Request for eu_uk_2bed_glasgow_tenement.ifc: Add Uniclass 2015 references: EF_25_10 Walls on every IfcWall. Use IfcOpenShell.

First a look at what the model holds.

```python
import ifcopenshell

model = ifcopenshell.open("eu_uk_2bed_glasgow_tenement.ifc")
print(model.schema)
print("classifications:", [c.Name for c in model.by_type("IfcClassification")])
for ifc_class in ("IfcDoor", "IfcRoof", "IfcStair", "IfcWall", "IfcWindow"):
    print(ifc_class, len(model.by_type(ifc_class)))
```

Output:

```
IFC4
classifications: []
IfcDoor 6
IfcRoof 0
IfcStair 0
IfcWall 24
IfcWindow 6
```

```python
import ifcopenshell
import ifcopenshell.api.classification

model = ifcopenshell.open("eu_uk_2bed_glasgow_tenement.ifc")

system = ifcopenshell.api.classification.add_classification(model, classification="Uniclass 2015")

codes = {
    "IfcWall": ("EF_25_10", "Walls"),
}
for ifc_class, (code, name) in codes.items():
    products = model.by_type(ifc_class)
    ifcopenshell.api.classification.add_reference(
        model, products=products, classification=system, identification=code, name=name
    )
    print(code, len(products))

model.write("eu_uk_2bed_glasgow_tenement_rev.ifc")
```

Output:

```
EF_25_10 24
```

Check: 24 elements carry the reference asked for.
